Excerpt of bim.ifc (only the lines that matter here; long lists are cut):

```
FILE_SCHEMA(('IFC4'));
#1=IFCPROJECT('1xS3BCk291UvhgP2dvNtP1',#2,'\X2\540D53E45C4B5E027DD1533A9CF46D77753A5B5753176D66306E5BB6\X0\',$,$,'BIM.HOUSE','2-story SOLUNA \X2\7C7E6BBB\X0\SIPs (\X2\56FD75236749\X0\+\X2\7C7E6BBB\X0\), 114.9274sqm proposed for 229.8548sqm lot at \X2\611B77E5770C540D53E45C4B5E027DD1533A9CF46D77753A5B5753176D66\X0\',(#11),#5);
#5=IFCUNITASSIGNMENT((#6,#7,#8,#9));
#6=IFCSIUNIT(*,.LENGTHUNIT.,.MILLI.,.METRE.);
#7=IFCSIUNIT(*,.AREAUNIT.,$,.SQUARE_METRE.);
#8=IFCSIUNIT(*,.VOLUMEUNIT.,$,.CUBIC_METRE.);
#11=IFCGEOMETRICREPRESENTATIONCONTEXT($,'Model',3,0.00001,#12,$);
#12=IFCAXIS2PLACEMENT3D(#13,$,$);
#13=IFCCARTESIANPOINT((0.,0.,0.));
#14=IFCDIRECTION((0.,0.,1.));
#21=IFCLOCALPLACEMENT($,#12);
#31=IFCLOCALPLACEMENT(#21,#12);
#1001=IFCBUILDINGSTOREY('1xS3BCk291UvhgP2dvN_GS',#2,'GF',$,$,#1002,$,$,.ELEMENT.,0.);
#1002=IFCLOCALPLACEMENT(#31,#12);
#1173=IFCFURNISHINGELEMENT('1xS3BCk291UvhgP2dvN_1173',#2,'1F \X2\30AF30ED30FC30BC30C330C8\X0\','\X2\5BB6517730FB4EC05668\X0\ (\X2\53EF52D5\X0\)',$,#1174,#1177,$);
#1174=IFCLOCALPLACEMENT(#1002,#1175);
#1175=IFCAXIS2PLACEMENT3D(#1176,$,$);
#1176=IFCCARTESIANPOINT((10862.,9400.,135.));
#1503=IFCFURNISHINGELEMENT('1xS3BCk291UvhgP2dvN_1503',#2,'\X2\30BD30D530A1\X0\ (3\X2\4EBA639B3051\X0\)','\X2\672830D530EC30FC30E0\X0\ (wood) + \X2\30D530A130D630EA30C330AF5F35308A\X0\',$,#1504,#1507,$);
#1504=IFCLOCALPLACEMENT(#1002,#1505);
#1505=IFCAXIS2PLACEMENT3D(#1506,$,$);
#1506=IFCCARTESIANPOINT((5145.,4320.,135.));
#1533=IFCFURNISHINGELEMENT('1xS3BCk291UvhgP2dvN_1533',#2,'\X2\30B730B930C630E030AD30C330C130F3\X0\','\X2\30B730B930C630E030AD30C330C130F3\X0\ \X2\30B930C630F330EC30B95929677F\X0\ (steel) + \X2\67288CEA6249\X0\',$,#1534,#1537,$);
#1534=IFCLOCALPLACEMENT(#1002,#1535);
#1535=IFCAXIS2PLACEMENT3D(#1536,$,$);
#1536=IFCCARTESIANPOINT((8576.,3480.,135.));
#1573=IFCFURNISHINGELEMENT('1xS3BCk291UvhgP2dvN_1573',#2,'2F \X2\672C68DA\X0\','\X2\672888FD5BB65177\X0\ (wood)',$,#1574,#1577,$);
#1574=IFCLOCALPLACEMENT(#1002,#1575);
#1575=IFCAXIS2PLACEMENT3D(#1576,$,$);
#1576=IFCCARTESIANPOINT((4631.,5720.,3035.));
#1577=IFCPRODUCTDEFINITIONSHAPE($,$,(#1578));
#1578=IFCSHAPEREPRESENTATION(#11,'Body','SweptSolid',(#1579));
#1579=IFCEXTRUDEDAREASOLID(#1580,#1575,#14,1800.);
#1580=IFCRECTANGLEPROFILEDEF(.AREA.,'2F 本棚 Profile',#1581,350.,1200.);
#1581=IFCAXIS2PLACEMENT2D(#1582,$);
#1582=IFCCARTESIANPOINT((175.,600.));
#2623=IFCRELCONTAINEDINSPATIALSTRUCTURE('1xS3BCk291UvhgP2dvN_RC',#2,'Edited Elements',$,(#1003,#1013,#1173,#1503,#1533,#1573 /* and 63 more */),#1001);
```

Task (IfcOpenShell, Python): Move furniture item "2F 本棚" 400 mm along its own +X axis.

```python
import ifcopenshell
import ifcopenshell.api.geometry
import ifcopenshell.util.placement

model = ifcopenshell.open("bim.ifc")

item = model.by_guid("1xS3BCk291UvhgP2dvN_1573")
matrix = ifcopenshell.util.placement.get_local_placement(item.ObjectPlacement)
matrix[:3, 3] += matrix[:3, 0] * 400.0
ifcopenshell.api.geometry.edit_object_placement(model, product=item, matrix=matrix, is_si=False)

print(ifcopenshell.util.placement.get_local_placement(item.ObjectPlacement).round(3) + 0.0)

model.write("bim_edited.ifc")
```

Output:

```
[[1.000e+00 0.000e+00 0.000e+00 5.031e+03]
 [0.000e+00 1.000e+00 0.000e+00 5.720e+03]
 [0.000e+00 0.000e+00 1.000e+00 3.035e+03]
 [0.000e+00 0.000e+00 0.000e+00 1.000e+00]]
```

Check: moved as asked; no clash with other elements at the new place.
